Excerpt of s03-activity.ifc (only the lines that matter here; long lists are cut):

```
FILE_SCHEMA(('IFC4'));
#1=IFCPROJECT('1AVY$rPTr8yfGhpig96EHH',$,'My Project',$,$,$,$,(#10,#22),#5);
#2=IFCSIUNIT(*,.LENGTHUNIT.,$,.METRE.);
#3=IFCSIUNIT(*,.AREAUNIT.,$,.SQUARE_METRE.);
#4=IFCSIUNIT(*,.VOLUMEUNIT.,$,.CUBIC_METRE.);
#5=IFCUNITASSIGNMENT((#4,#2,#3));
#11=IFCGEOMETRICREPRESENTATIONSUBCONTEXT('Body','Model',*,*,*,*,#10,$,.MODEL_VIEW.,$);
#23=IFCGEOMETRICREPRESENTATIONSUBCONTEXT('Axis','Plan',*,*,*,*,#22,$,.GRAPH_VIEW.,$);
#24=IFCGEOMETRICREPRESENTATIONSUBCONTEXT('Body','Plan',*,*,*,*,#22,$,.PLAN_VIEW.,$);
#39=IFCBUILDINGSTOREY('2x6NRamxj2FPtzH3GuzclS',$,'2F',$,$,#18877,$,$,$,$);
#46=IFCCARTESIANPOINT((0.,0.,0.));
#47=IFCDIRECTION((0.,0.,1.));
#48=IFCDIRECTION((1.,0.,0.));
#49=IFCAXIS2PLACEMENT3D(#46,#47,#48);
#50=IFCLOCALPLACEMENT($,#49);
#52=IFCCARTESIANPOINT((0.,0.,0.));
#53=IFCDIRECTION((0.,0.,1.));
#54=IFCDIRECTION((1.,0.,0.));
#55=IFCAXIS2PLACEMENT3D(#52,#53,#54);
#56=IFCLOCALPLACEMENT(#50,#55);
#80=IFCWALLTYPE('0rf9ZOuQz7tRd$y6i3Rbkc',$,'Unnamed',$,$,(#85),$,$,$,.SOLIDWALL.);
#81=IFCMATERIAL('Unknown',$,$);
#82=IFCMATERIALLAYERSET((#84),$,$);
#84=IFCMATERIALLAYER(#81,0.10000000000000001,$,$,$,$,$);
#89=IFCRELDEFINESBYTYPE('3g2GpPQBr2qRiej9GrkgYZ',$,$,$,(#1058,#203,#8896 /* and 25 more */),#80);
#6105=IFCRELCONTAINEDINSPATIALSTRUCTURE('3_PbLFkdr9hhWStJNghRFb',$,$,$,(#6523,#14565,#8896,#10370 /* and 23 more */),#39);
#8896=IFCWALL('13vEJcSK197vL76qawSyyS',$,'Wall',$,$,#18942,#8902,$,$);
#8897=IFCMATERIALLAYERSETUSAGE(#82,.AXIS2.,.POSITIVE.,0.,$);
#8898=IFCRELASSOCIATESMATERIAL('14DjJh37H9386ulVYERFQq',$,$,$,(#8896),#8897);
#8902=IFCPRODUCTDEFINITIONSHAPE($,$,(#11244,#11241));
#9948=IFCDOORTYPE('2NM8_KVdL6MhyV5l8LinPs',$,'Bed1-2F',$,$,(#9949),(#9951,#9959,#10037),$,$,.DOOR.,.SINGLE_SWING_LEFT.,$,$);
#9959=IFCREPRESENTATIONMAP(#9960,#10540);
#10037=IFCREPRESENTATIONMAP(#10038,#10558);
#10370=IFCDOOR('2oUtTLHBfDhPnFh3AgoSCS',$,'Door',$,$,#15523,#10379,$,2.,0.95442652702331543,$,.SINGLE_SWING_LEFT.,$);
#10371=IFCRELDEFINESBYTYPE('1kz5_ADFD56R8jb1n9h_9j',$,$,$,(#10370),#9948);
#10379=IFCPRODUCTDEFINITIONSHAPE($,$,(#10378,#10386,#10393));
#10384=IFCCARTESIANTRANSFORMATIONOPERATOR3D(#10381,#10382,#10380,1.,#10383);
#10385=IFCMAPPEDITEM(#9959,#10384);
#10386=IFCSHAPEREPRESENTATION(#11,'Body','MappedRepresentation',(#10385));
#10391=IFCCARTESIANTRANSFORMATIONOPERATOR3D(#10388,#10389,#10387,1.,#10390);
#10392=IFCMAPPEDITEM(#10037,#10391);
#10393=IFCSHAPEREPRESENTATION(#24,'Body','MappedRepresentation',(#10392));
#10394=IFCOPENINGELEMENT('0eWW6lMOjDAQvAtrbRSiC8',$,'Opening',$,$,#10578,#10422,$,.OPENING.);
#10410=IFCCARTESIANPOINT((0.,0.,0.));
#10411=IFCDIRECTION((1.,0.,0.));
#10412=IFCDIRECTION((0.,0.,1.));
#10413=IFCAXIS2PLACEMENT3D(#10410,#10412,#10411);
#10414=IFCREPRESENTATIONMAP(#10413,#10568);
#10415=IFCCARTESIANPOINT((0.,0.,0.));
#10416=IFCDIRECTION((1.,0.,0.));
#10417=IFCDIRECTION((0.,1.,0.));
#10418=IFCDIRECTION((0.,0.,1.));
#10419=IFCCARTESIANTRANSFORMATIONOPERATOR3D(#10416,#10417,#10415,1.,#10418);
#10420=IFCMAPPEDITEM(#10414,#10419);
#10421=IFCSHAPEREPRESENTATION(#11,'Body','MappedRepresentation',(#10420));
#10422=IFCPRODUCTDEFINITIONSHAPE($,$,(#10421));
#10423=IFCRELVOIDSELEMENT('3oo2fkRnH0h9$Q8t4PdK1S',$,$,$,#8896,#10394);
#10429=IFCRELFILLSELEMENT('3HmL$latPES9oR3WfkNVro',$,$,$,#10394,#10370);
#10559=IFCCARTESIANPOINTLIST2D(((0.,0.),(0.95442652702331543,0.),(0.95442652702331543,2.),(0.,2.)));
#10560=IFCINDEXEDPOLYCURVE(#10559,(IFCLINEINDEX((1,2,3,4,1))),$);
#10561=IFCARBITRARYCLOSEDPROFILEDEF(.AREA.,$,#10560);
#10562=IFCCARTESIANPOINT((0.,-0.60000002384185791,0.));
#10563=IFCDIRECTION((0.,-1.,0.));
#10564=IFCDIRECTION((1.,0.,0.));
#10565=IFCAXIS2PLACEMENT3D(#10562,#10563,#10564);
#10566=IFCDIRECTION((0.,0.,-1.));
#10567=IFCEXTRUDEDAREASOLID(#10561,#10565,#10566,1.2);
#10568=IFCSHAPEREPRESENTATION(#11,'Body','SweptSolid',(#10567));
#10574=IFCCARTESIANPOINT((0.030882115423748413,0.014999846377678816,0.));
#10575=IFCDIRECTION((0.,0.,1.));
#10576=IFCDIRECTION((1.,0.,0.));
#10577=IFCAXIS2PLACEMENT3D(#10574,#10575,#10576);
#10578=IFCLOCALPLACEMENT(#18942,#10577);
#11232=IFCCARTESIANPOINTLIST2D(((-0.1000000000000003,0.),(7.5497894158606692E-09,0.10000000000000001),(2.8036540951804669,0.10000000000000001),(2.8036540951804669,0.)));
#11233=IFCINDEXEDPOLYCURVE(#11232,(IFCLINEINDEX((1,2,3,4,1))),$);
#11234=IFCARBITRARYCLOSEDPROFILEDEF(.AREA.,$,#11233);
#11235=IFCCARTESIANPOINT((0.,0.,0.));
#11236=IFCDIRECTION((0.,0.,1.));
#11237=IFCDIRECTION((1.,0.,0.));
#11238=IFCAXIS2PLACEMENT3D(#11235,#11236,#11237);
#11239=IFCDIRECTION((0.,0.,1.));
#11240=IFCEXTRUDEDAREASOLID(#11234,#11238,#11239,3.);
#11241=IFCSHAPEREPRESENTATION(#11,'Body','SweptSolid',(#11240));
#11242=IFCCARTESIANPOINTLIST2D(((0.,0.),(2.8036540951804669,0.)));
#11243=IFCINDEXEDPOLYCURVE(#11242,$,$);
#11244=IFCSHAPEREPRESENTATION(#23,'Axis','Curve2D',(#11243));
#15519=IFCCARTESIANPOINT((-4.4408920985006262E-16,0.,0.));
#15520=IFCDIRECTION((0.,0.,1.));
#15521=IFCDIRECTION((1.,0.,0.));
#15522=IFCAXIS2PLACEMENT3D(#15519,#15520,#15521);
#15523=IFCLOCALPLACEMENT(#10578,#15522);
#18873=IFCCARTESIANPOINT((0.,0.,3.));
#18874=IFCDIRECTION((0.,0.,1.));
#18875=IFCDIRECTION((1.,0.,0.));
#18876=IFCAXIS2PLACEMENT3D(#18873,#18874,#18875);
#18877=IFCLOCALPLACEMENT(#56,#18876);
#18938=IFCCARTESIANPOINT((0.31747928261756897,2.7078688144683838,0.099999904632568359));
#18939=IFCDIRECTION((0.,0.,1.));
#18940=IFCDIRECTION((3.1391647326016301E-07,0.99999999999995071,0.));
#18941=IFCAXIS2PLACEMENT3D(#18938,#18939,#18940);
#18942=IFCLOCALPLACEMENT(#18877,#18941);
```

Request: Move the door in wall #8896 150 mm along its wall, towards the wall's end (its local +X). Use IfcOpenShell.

```python
import ifcopenshell
import ifcopenshell.api.geometry
import ifcopenshell.util.placement
import ifcopenshell.util.unit

model = ifcopenshell.open("s03-activity.ifc")
unit_scale = ifcopenshell.util.unit.calculate_unit_scale(model)

door = model.by_guid("2oUtTLHBfDhPnFh3AgoSCS")
opening = door.FillsVoids[0].RelatingOpeningElement
wall = opening.VoidsElements[0].RelatingBuildingElement

wall_matrix = ifcopenshell.util.placement.get_local_placement(wall.ObjectPlacement)
shift = wall_matrix[:3, 0] * 0.15 / unit_scale
before = ifcopenshell.util.placement.get_local_placement(door.ObjectPlacement)[:3, 3].copy()

# The door is placed relative to its opening, so it follows when the opening moves.
matrix = ifcopenshell.util.placement.get_local_placement(opening.ObjectPlacement)
matrix[:3, 3] += shift
ifcopenshell.api.geometry.edit_object_placement(
    model, product=opening, matrix=matrix, is_si=False, should_transform_children=True
)

after = ifcopenshell.util.placement.get_local_placement(door.ObjectPlacement)[:3, 3]
print("door moved by", (after - before).round(3) + 0.0)

model.write("s03-activity_v2.ifc")
```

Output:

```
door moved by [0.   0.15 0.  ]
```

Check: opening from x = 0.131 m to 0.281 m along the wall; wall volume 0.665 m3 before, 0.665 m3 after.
